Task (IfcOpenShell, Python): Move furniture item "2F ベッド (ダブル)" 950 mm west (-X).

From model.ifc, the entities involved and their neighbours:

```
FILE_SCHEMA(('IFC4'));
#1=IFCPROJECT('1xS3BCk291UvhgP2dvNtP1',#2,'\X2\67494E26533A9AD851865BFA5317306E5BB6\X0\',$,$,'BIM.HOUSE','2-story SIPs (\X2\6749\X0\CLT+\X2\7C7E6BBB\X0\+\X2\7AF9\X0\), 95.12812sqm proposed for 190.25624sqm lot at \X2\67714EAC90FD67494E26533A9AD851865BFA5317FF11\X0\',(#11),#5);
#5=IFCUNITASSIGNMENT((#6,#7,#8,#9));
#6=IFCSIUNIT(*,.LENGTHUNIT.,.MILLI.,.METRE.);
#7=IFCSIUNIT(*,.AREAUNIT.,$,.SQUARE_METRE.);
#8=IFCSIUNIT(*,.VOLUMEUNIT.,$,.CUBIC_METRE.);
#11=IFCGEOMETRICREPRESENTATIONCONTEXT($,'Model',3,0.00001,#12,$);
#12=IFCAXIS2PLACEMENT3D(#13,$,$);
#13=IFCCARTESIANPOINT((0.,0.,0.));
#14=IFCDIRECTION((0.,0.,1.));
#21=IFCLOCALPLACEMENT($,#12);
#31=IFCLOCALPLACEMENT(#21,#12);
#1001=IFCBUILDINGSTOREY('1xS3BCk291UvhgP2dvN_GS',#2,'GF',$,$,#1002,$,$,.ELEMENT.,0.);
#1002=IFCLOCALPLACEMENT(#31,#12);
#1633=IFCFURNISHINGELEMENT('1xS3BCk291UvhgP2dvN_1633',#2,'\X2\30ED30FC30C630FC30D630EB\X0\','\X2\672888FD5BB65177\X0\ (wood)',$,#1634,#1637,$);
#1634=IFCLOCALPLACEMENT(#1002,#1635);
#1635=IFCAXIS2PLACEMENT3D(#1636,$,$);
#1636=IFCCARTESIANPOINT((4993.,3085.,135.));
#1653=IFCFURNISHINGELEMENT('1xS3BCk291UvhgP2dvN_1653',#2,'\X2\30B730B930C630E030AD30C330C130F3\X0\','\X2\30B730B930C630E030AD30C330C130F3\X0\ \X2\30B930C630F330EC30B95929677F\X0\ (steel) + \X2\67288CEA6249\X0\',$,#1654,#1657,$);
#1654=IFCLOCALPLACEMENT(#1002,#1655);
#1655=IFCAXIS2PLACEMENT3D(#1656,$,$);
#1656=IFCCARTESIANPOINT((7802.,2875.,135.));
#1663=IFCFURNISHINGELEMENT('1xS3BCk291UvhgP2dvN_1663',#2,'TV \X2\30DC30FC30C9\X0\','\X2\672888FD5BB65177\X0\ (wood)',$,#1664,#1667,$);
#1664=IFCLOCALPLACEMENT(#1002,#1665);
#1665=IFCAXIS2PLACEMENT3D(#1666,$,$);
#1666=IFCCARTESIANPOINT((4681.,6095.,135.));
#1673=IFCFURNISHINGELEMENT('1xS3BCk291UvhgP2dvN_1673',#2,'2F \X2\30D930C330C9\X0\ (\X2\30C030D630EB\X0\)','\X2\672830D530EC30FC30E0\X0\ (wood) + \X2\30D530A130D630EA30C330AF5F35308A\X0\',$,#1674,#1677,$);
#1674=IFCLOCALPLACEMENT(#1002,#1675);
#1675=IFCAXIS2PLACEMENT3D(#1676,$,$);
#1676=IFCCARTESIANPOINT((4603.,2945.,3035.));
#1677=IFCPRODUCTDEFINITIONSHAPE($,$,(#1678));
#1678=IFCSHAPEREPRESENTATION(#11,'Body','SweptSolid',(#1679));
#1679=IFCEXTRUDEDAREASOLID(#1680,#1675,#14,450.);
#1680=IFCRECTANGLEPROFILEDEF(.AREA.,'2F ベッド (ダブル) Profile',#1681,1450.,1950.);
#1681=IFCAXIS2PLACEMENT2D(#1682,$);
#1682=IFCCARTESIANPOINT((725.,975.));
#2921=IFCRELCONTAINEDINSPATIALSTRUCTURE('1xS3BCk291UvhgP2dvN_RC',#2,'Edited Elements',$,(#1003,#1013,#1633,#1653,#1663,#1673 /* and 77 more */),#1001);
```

```python
import ifcopenshell
import ifcopenshell.api.geometry
import ifcopenshell.util.placement
import ifcopenshell.util.unit

model = ifcopenshell.open("model.ifc")
unit_scale = ifcopenshell.util.unit.calculate_unit_scale(model)

item = model.by_id(1673)
matrix = ifcopenshell.util.placement.get_local_placement(item.ObjectPlacement)
matrix[0, 3] -= 0.95 / unit_scale
ifcopenshell.api.geometry.edit_object_placement(model, product=item, matrix=matrix, is_si=False)

print(ifcopenshell.util.placement.get_local_placement(item.ObjectPlacement).round(3) + 0.0)

model.write("model_updated.ifc")
```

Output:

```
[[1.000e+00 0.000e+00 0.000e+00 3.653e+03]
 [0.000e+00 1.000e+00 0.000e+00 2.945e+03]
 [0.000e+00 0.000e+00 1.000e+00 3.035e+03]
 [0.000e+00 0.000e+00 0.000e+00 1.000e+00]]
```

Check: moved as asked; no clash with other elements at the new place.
